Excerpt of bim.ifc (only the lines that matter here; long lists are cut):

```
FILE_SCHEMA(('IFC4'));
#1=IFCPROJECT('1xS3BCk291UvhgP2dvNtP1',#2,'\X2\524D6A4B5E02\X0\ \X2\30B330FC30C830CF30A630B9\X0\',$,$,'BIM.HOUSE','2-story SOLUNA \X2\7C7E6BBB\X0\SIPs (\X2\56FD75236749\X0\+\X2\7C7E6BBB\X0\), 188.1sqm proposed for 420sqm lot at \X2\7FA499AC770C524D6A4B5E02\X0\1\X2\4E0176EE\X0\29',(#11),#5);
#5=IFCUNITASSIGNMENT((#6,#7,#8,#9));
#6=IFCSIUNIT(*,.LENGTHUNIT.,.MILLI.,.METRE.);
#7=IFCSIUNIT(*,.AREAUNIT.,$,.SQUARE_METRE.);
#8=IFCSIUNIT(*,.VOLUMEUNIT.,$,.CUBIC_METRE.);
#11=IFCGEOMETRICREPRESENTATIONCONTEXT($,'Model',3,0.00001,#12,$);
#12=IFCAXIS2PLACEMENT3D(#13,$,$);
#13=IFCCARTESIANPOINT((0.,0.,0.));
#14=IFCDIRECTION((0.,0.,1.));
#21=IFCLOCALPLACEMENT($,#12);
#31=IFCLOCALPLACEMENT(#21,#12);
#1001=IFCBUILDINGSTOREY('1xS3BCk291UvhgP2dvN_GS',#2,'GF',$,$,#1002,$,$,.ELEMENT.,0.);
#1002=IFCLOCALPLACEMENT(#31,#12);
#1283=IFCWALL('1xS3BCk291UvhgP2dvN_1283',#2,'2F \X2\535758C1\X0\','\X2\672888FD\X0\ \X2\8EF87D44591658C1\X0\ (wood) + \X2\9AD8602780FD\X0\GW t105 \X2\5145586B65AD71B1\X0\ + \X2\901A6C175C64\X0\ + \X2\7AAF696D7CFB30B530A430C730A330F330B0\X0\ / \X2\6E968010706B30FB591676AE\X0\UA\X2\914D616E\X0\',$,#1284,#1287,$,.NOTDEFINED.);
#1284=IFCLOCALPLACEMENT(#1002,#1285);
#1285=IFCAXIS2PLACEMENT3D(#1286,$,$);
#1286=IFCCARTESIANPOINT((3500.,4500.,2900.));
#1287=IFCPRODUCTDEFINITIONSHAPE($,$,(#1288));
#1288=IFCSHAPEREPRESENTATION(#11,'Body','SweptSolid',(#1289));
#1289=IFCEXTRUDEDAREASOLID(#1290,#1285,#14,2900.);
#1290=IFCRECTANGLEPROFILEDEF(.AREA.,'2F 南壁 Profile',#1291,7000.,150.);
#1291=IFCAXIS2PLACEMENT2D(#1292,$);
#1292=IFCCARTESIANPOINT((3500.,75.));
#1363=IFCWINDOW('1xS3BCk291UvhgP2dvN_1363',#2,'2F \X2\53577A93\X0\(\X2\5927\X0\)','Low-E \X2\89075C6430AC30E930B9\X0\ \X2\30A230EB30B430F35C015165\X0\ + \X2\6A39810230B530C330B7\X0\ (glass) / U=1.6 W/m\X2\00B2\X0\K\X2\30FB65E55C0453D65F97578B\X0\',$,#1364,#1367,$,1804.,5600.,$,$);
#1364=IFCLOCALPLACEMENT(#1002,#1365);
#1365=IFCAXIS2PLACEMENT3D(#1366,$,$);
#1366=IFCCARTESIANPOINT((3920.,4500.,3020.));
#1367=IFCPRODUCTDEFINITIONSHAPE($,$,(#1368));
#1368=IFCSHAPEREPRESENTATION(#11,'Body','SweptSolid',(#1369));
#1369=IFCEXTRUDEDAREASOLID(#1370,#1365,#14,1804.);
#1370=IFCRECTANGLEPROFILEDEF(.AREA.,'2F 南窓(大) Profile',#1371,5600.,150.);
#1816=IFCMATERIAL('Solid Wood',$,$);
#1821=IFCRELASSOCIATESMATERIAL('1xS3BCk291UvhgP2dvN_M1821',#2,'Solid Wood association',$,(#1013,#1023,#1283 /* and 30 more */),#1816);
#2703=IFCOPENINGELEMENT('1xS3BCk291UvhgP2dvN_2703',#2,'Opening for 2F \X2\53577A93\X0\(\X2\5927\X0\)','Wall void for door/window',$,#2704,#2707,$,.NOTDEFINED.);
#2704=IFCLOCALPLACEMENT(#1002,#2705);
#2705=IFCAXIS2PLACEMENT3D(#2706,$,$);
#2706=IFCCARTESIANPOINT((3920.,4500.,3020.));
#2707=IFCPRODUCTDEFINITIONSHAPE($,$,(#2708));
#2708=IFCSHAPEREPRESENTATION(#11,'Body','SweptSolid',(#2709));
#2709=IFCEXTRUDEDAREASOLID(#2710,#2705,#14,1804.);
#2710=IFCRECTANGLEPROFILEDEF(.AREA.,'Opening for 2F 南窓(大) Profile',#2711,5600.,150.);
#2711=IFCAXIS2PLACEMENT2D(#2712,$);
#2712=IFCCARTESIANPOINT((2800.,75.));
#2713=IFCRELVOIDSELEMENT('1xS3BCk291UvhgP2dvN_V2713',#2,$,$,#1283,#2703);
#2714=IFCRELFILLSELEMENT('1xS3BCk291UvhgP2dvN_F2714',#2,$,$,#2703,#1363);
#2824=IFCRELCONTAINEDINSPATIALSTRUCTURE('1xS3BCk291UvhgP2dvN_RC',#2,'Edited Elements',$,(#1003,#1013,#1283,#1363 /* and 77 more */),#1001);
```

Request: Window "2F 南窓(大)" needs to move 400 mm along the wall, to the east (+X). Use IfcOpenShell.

```python
import ifcopenshell
import ifcopenshell.api.geometry
import ifcopenshell.util.placement
import ifcopenshell.util.unit

model = ifcopenshell.open("bim.ifc")
unit_scale = ifcopenshell.util.unit.calculate_unit_scale(model)

window = model.by_id(1363)
opening = window.FillsVoids[0].RelatingOpeningElement
wall = opening.VoidsElements[0].RelatingBuildingElement

wall_matrix = ifcopenshell.util.placement.get_local_placement(wall.ObjectPlacement)
shift = wall_matrix[:3, 0] * 0.4 / unit_scale
before = ifcopenshell.util.placement.get_local_placement(window.ObjectPlacement)[:3, 3].copy()

# The window is not placed relative to its opening, so move both.
for product in (opening, window):
    matrix = ifcopenshell.util.placement.get_local_placement(product.ObjectPlacement)
    matrix[:3, 3] += shift
    ifcopenshell.api.geometry.edit_object_placement(model, product=product, matrix=matrix, is_si=False)

after = ifcopenshell.util.placement.get_local_placement(window.ObjectPlacement)[:3, 3]
print("window moved by", (after - before).round(3) + 0.0)

model.write("bim_v2.ifc")
```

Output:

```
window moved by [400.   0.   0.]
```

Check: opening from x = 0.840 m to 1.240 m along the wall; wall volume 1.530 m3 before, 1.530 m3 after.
